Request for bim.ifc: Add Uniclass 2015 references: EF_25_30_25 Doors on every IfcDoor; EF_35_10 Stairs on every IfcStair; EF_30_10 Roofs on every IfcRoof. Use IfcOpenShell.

First a look at what the model holds.

```python
import ifcopenshell

model = ifcopenshell.open("bim.ifc")
print(model.schema)
print("classifications:", [c.Name for c in model.by_type("IfcClassification")])
for ifc_class in ("IfcDoor", "IfcRoof", "IfcStair", "IfcWall", "IfcWindow"):
    print(ifc_class, len(model.by_type(ifc_class)))
```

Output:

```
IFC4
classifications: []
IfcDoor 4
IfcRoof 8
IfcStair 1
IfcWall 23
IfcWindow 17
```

```python
import ifcopenshell
import ifcopenshell.api.classification

model = ifcopenshell.open("bim.ifc")

system = ifcopenshell.api.classification.add_classification(model, classification="Uniclass 2015")

codes = {
    "IfcDoor": ("EF_25_30_25", "Doors"),
    "IfcStair": ("EF_35_10", "Stairs"),
    "IfcRoof": ("EF_30_10", "Roofs"),
}
for ifc_class, (code, name) in codes.items():
    products = model.by_type(ifc_class)
    ifcopenshell.api.classification.add_reference(
        model, products=products, classification=system, identification=code, name=name
    )
    print(code, len(products))

model.write("bim_rev.ifc")
```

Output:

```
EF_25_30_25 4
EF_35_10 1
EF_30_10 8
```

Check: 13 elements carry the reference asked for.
